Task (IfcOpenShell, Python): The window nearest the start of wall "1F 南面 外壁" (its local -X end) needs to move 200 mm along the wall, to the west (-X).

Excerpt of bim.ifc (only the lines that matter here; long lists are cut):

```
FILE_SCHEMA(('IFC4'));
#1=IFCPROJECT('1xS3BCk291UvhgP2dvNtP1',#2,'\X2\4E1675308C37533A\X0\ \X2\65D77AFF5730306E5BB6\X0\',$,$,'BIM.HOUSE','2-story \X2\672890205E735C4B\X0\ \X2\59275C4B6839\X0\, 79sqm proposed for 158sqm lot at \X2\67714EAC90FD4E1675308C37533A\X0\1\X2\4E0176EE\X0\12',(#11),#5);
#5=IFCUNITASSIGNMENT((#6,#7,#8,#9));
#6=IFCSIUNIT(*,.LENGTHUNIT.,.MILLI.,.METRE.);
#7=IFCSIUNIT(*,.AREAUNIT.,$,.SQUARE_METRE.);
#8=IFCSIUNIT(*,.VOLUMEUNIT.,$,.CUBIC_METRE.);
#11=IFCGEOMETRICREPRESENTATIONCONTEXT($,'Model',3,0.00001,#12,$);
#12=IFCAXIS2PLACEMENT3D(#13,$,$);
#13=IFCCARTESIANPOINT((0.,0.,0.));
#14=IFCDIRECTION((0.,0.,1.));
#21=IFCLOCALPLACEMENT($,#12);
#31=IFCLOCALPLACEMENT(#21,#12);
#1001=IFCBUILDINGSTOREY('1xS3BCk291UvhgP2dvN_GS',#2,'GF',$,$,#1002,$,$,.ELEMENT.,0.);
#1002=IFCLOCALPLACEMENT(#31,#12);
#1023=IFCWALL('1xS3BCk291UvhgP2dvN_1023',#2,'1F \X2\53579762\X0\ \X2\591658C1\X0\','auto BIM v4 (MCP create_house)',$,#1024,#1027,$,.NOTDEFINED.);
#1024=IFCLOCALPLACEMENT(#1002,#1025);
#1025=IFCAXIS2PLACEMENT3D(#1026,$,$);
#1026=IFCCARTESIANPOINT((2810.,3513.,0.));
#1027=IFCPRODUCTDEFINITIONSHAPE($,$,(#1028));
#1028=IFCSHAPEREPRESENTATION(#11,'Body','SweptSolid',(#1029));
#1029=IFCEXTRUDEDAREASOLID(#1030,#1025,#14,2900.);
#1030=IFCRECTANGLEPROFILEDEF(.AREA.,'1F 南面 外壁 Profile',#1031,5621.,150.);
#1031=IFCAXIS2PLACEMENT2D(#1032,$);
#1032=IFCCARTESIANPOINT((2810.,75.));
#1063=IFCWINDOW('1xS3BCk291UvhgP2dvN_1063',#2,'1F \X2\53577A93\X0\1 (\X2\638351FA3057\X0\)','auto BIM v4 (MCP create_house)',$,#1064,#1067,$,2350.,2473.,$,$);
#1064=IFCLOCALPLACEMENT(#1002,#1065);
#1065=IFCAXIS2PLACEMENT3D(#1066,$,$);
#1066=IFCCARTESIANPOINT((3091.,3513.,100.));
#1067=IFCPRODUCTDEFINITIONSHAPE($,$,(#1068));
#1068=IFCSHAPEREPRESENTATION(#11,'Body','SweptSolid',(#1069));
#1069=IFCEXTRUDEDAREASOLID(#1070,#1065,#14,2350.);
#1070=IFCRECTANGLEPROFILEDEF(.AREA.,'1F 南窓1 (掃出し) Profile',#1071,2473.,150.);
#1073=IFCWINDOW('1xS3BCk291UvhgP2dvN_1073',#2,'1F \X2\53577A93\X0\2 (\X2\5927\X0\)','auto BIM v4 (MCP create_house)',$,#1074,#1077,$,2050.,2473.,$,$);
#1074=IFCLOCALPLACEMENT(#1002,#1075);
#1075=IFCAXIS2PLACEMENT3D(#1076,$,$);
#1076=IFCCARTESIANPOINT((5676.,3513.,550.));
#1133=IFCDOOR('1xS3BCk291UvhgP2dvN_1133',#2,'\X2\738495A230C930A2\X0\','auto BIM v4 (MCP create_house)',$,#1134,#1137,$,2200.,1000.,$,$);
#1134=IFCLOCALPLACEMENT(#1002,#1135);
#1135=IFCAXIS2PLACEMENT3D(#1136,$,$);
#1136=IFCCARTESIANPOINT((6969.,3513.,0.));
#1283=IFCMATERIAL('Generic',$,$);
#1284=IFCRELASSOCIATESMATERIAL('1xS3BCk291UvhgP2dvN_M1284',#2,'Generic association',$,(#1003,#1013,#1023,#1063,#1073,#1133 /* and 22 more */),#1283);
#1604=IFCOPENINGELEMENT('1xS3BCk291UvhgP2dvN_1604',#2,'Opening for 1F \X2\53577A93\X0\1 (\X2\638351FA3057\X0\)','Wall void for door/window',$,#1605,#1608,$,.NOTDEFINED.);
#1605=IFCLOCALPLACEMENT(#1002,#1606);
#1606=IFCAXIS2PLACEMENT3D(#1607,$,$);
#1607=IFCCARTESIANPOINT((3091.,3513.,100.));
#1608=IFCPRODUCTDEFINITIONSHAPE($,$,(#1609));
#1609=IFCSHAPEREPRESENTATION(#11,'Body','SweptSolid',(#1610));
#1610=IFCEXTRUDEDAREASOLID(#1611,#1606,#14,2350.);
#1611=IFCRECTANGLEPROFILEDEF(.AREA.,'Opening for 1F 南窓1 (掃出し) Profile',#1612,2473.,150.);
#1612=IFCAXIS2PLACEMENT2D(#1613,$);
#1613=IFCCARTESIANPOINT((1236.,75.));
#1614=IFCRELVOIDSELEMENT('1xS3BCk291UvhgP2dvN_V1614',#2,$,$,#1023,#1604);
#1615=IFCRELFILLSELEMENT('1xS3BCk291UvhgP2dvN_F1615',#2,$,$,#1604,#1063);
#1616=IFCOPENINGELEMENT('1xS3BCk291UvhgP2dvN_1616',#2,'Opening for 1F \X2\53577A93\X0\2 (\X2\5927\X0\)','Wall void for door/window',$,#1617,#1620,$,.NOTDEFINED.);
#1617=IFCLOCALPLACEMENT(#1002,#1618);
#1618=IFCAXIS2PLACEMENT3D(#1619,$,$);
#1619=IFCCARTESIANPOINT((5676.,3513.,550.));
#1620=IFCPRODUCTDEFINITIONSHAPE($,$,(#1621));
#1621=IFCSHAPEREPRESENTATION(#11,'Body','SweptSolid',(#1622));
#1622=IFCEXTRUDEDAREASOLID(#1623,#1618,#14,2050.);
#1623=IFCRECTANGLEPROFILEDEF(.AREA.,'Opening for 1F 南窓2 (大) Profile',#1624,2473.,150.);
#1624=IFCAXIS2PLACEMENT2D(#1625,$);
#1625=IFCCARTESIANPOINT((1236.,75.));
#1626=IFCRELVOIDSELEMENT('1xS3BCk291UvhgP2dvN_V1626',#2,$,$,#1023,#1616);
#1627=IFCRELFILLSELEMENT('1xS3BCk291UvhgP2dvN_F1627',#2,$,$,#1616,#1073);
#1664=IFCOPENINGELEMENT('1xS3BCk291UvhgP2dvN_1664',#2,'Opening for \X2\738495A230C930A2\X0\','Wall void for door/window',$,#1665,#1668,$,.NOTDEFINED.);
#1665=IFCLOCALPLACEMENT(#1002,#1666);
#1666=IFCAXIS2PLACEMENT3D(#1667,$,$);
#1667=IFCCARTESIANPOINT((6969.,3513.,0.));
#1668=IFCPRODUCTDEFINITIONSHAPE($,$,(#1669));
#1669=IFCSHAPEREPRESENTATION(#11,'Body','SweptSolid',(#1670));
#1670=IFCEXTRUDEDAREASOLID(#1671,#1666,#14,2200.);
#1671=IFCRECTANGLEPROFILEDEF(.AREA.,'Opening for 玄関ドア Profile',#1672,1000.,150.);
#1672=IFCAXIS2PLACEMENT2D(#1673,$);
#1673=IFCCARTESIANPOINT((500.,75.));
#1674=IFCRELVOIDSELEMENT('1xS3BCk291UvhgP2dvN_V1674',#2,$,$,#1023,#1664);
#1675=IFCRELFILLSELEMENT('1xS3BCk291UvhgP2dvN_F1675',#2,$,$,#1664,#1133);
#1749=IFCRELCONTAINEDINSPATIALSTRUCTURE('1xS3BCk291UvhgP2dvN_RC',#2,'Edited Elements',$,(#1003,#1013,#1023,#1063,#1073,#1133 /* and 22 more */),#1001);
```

```python
import ifcopenshell
import ifcopenshell.api.geometry
import ifcopenshell.util.placement
import ifcopenshell.util.unit

model = ifcopenshell.open("bim.ifc")
unit_scale = ifcopenshell.util.unit.calculate_unit_scale(model)

window = model.by_guid("1xS3BCk291UvhgP2dvN_1063")
opening = window.FillsVoids[0].RelatingOpeningElement
wall = opening.VoidsElements[0].RelatingBuildingElement

wall_matrix = ifcopenshell.util.placement.get_local_placement(wall.ObjectPlacement)
shift = wall_matrix[:3, 0] * -0.2 / unit_scale
before = ifcopenshell.util.placement.get_local_placement(window.ObjectPlacement)[:3, 3].copy()

# The window is not placed relative to its opening, so move both.
for product in (opening, window):
    matrix = ifcopenshell.util.placement.get_local_placement(product.ObjectPlacement)
    matrix[:3, 3] += shift
    ifcopenshell.api.geometry.edit_object_placement(model, product=product, matrix=matrix, is_si=False)

after = ifcopenshell.util.placement.get_local_placement(window.ObjectPlacement)[:3, 3]
print("window moved by", (after - before).round(3) + 0.0)

model.write("bim_updated.ifc")
```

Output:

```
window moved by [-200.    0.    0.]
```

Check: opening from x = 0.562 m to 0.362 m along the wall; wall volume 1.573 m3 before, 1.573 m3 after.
